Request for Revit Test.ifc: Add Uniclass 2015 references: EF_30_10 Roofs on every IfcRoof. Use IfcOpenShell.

First a look at what the model holds.

```python
import ifcopenshell

model = ifcopenshell.open("Revit Test.ifc")
print(model.schema)
print("classifications:", [c.Name for c in model.by_type("IfcClassification")])
for ifc_class in ("IfcDoor", "IfcRoof", "IfcStair", "IfcWall", "IfcWindow"):
    print(ifc_class, len(model.by_type(ifc_class)))
```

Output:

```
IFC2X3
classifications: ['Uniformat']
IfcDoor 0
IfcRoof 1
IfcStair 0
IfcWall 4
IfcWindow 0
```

```python
import ifcopenshell
import ifcopenshell.api.classification

model = ifcopenshell.open("Revit Test.ifc")

# IFC2X3 requires Source and Edition and has no link from the project to the system.
system = model.create_entity("IfcClassification", Source="NBS", Edition="2015", Name="Uniclass 2015")

codes = {
    "IfcRoof": ("EF_30_10", "Roofs"),
}
for ifc_class, (code, name) in codes.items():
    products = model.by_type(ifc_class)
    ifcopenshell.api.classification.add_reference(
        model, products=products, classification=system, identification=code, name=name
    )
    print(code, len(products))

model.write("Revit Test-out.ifc")
```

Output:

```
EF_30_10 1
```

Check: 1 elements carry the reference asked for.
